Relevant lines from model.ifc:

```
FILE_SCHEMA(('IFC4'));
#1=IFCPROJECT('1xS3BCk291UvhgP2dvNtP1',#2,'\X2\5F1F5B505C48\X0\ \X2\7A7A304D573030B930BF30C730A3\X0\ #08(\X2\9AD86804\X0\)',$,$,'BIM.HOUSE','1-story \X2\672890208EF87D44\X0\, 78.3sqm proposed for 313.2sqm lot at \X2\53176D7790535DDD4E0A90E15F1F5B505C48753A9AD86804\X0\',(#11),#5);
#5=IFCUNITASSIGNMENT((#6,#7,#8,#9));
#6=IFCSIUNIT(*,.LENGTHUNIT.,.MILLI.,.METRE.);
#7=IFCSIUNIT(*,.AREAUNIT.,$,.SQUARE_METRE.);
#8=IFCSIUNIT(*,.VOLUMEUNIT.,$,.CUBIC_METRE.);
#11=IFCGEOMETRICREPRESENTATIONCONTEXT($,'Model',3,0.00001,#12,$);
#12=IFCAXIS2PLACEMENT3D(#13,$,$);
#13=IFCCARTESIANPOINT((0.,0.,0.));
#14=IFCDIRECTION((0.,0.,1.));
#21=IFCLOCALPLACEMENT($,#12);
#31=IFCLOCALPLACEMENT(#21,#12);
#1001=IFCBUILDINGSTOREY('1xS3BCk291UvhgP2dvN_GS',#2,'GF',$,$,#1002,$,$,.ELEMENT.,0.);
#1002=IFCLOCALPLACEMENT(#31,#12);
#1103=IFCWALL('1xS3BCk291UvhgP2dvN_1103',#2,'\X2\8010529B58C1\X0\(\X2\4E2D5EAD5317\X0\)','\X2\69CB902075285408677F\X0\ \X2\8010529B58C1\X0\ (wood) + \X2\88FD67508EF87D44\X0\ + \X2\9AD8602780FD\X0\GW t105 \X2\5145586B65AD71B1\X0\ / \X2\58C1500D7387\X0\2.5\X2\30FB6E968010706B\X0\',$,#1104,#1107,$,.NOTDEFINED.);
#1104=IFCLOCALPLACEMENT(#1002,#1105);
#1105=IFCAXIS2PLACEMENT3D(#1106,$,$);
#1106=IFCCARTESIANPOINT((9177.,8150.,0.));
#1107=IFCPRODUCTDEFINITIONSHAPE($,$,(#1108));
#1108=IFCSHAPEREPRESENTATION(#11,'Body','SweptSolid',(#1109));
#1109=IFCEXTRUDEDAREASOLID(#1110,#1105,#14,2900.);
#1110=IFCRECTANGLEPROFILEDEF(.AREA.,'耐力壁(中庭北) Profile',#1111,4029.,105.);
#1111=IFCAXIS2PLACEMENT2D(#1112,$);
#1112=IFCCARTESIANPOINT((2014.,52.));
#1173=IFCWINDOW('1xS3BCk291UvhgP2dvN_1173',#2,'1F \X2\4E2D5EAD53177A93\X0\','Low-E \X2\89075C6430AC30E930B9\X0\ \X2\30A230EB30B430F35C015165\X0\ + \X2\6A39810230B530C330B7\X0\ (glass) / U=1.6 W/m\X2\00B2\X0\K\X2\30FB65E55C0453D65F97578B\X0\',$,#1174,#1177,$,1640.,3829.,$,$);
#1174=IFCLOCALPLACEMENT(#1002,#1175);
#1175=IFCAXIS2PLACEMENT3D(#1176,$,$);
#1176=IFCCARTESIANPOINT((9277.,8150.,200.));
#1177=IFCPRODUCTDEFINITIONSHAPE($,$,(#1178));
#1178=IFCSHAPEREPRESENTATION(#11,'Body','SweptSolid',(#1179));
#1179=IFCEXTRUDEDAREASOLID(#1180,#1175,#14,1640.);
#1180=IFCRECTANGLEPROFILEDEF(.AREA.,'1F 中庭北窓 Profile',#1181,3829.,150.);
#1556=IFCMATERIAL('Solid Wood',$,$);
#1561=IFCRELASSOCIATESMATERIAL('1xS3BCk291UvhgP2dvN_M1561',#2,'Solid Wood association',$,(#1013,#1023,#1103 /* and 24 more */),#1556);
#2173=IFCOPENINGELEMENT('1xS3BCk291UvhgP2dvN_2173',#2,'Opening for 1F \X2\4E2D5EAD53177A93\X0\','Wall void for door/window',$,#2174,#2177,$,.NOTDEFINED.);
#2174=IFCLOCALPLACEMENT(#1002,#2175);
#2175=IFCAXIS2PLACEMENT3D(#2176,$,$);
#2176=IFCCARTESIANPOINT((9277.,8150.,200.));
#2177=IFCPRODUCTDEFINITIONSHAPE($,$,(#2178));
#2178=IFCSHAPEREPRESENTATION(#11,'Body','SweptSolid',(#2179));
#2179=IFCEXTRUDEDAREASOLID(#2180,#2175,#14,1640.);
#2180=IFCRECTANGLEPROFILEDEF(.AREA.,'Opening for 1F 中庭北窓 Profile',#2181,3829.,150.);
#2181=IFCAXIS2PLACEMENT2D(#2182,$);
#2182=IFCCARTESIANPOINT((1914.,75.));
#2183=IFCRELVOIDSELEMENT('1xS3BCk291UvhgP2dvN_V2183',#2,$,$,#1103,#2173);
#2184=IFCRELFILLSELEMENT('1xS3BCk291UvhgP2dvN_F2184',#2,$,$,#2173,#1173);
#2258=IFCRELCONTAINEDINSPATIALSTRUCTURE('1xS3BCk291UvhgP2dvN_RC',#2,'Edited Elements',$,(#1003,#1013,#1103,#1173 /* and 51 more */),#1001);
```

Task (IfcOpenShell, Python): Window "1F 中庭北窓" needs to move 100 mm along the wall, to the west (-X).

```python
import ifcopenshell
import ifcopenshell.api.geometry
import ifcopenshell.util.placement

model = ifcopenshell.open("model.ifc")

window = model.by_guid("1xS3BCk291UvhgP2dvN_1173")
opening = window.FillsVoids[0].RelatingOpeningElement
wall = opening.VoidsElements[0].RelatingBuildingElement

wall_matrix = ifcopenshell.util.placement.get_local_placement(wall.ObjectPlacement)
shift = wall_matrix[:3, 0] * -100.0
before = ifcopenshell.util.placement.get_local_placement(window.ObjectPlacement)[:3, 3].copy()

# The window is not placed relative to its opening, so move both.
for product in (opening, window):
    matrix = ifcopenshell.util.placement.get_local_placement(product.ObjectPlacement)
    matrix[:3, 3] += shift
    ifcopenshell.api.geometry.edit_object_placement(model, product=product, matrix=matrix, is_si=False)

after = ifcopenshell.util.placement.get_local_placement(window.ObjectPlacement)[:3, 3]
print("window moved by", (after - before).round(3) + 0.0)

model.write("model_rev.ifc")
```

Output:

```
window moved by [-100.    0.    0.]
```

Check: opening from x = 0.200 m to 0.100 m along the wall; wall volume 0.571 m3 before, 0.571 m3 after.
